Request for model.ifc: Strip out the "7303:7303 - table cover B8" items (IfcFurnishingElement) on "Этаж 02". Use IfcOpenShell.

First a look at what the model holds.

```python
import ifcopenshell
import ifcopenshell.util.element

model = ifcopenshell.open("model.ifc")
print(model.schema)
storey = next(s for s in model.by_type("IfcBuildingStorey") if s.Name == "Этаж 02")
furniture = [e for e in ifcopenshell.util.element.get_decomposition(storey) if e.is_a("IfcFurnishingElement")]
seen = {}
for e in furniture:
    element_type = ifcopenshell.util.element.get_type(e)
    name = element_type.Name if element_type not in (None, e) else None
    seen[name] = seen.get(name, 0) + 1
for name, count in sorted(seen.items(), key=str):
    print(count, "x", name)
```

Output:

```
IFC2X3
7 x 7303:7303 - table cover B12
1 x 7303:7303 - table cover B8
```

```python
import ifcopenshell
import ifcopenshell.api.root
import ifcopenshell.util.element

model = ifcopenshell.open("model.ifc")

storey = next(s for s in model.by_type("IfcBuildingStorey") if s.Name == "Этаж 02")
furniture = [e for e in ifcopenshell.util.element.get_decomposition(storey) if e.is_a("IfcFurnishingElement")]
targets = [e for e in furniture if (t := ifcopenshell.util.element.get_type(e)) not in (None, e) and t.Name == "7303:7303 - table cover B8"]

for e in targets:
    ifcopenshell.api.root.remove_product(model, product=e)
print(len(targets), "removed")

model.write("model_edited.ifc")
```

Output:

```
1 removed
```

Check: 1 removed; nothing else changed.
